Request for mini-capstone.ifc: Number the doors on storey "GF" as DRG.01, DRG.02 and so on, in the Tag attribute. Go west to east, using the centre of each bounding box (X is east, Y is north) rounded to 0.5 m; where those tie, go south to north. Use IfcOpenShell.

First a look at what the model holds.

```python
import ifcopenshell
import ifcopenshell.util.element
import ifcopenshell.util.placement

model = ifcopenshell.open("mini-capstone.ifc")
print(model.schema)
storey = next(s for s in model.by_type("IfcBuildingStorey") if s.Name == "GF")
doors = [e for e in ifcopenshell.util.element.get_decomposition(storey) if e.is_a("IfcDoor")]
for e in sorted(doors, key=lambda e: e.id()):
    origin = ifcopenshell.util.placement.get_local_placement(e.ObjectPlacement)[:3, 3]
    print(e.id(), e.Tag, e.Name, origin.round(2) + 0.0, sep=" | ")
```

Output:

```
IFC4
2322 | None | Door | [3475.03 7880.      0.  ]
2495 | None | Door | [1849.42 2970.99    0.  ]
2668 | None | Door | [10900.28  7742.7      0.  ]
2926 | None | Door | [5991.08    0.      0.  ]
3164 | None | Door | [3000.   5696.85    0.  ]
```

```python
import ifcopenshell
import ifcopenshell.geom
import ifcopenshell.util.element
import ifcopenshell.util.shape

model = ifcopenshell.open("mini-capstone.ifc")
settings = ifcopenshell.geom.settings()
settings.set("use-world-coords", True)


def centre(element):
    shape = ifcopenshell.geom.create_shape(settings, element)
    return ifcopenshell.util.shape.get_bbox_centroid(shape.geometry)


storey = next(s for s in model.by_type("IfcBuildingStorey") if s.Name == "GF")
doors = [e for e in ifcopenshell.util.element.get_decomposition(storey) if e.is_a("IfcDoor")]

# Insertion points can sit at a corner or the storey origin, so sort by the geometry (in metres).
centres = {e: centre(e) for e in doors}
doors.sort(key=lambda e: (round(centres[e][0] / 0.5), centres[e][1]))

for i, e in enumerate(doors, start=1):
    number = f"DRG.{i:02d}"
    e.Tag = number
    print(e.id(), number)

model.write("mini-capstone-out.ifc")
```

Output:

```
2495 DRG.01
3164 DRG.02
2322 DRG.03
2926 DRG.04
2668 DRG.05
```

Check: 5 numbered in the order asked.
